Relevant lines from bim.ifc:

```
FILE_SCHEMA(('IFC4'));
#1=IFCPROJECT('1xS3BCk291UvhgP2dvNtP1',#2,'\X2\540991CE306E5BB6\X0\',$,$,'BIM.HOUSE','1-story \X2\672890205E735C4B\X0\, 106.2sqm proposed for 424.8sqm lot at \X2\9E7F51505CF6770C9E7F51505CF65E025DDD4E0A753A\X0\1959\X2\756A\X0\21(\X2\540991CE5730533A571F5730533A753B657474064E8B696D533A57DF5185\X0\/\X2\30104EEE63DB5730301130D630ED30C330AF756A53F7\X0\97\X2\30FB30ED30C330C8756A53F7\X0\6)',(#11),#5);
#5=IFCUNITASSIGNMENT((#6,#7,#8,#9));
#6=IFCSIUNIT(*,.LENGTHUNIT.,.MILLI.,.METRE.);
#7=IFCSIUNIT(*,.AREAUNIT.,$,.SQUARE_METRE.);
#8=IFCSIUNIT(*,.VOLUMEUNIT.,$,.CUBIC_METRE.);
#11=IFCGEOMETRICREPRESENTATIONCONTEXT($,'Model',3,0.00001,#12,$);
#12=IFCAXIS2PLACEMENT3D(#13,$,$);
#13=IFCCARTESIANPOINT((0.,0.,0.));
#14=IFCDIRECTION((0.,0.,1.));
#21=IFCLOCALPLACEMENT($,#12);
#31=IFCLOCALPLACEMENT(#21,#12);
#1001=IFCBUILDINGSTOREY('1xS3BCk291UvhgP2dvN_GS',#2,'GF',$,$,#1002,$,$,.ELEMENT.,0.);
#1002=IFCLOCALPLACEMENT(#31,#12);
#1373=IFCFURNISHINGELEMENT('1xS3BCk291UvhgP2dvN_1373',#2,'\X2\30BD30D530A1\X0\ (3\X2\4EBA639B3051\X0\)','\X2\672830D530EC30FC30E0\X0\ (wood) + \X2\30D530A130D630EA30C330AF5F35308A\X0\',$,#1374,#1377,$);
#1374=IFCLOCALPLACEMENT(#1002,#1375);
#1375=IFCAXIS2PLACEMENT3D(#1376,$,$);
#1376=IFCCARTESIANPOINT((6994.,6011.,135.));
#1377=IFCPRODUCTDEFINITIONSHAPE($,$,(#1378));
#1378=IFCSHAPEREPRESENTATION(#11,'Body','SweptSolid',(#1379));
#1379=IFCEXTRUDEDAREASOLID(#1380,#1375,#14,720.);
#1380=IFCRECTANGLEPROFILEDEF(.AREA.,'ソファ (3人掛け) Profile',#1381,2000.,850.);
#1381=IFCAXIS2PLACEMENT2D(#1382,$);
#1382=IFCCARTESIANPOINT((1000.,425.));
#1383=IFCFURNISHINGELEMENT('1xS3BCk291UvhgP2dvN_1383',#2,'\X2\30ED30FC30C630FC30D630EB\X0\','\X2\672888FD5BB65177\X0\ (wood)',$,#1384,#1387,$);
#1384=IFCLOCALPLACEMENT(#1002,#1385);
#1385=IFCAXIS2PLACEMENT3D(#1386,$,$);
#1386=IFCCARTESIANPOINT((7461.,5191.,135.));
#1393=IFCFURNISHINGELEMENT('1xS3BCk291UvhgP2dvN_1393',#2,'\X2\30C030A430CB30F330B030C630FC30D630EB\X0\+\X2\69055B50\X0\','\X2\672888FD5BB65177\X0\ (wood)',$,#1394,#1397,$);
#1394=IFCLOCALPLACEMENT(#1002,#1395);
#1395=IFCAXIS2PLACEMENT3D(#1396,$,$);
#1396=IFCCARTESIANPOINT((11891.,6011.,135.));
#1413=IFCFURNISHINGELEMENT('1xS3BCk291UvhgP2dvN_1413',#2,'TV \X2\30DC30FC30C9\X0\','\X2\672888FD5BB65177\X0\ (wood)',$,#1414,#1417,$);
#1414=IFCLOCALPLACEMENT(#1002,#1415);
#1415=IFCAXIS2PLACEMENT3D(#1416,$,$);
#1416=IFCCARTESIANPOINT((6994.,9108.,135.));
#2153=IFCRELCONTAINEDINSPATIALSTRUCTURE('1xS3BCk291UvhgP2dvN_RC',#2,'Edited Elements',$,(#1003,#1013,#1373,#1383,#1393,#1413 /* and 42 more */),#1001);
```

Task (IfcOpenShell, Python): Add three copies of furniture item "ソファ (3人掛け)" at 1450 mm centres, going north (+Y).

```python
import numpy as np
import ifcopenshell
import ifcopenshell.api.geometry
import ifcopenshell.api.root
import ifcopenshell.util.element
import ifcopenshell.util.placement
import ifcopenshell.util.unit

model = ifcopenshell.open("bim.ifc")
unit_scale = ifcopenshell.util.unit.calculate_unit_scale(model)


def reuse_history(source, copy):
    """copy_class also copies each property set's owner history, people and application; keep the originals."""
    for rel in copy.IsDefinedBy:
        if rel.is_a("IfcRelDefinesByProperties") and (history := rel.RelatingPropertyDefinition.OwnerHistory):
            rel.RelatingPropertyDefinition.OwnerHistory = source.OwnerHistory
            ifcopenshell.util.element.remove_deep2(model, history)


source = model.by_guid("1xS3BCk291UvhgP2dvN_1373")
base = ifcopenshell.util.placement.get_local_placement(source.ObjectPlacement)
step = np.array([0.0, 1.0, 0.0]) * 1.45 / unit_scale

for i in range(1, 4):
    copy = ifcopenshell.api.root.copy_class(model, product=source)
    copy.Representation = ifcopenshell.util.element.copy_deep(
        model, source.Representation, exclude=["IfcGeometricRepresentationContext", "IfcRepresentationMap"]
    )
    reuse_history(source, copy)
    matrix = base.copy()
    matrix[:3, 3] += i * step
    print("added at", matrix[:3, 3].round(3) + 0.0)
    ifcopenshell.api.geometry.edit_object_placement(model, product=copy, matrix=matrix, is_si=False)

model.write("bim_v2.ifc")
```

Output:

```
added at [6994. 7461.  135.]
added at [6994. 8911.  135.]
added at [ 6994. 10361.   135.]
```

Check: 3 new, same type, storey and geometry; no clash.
